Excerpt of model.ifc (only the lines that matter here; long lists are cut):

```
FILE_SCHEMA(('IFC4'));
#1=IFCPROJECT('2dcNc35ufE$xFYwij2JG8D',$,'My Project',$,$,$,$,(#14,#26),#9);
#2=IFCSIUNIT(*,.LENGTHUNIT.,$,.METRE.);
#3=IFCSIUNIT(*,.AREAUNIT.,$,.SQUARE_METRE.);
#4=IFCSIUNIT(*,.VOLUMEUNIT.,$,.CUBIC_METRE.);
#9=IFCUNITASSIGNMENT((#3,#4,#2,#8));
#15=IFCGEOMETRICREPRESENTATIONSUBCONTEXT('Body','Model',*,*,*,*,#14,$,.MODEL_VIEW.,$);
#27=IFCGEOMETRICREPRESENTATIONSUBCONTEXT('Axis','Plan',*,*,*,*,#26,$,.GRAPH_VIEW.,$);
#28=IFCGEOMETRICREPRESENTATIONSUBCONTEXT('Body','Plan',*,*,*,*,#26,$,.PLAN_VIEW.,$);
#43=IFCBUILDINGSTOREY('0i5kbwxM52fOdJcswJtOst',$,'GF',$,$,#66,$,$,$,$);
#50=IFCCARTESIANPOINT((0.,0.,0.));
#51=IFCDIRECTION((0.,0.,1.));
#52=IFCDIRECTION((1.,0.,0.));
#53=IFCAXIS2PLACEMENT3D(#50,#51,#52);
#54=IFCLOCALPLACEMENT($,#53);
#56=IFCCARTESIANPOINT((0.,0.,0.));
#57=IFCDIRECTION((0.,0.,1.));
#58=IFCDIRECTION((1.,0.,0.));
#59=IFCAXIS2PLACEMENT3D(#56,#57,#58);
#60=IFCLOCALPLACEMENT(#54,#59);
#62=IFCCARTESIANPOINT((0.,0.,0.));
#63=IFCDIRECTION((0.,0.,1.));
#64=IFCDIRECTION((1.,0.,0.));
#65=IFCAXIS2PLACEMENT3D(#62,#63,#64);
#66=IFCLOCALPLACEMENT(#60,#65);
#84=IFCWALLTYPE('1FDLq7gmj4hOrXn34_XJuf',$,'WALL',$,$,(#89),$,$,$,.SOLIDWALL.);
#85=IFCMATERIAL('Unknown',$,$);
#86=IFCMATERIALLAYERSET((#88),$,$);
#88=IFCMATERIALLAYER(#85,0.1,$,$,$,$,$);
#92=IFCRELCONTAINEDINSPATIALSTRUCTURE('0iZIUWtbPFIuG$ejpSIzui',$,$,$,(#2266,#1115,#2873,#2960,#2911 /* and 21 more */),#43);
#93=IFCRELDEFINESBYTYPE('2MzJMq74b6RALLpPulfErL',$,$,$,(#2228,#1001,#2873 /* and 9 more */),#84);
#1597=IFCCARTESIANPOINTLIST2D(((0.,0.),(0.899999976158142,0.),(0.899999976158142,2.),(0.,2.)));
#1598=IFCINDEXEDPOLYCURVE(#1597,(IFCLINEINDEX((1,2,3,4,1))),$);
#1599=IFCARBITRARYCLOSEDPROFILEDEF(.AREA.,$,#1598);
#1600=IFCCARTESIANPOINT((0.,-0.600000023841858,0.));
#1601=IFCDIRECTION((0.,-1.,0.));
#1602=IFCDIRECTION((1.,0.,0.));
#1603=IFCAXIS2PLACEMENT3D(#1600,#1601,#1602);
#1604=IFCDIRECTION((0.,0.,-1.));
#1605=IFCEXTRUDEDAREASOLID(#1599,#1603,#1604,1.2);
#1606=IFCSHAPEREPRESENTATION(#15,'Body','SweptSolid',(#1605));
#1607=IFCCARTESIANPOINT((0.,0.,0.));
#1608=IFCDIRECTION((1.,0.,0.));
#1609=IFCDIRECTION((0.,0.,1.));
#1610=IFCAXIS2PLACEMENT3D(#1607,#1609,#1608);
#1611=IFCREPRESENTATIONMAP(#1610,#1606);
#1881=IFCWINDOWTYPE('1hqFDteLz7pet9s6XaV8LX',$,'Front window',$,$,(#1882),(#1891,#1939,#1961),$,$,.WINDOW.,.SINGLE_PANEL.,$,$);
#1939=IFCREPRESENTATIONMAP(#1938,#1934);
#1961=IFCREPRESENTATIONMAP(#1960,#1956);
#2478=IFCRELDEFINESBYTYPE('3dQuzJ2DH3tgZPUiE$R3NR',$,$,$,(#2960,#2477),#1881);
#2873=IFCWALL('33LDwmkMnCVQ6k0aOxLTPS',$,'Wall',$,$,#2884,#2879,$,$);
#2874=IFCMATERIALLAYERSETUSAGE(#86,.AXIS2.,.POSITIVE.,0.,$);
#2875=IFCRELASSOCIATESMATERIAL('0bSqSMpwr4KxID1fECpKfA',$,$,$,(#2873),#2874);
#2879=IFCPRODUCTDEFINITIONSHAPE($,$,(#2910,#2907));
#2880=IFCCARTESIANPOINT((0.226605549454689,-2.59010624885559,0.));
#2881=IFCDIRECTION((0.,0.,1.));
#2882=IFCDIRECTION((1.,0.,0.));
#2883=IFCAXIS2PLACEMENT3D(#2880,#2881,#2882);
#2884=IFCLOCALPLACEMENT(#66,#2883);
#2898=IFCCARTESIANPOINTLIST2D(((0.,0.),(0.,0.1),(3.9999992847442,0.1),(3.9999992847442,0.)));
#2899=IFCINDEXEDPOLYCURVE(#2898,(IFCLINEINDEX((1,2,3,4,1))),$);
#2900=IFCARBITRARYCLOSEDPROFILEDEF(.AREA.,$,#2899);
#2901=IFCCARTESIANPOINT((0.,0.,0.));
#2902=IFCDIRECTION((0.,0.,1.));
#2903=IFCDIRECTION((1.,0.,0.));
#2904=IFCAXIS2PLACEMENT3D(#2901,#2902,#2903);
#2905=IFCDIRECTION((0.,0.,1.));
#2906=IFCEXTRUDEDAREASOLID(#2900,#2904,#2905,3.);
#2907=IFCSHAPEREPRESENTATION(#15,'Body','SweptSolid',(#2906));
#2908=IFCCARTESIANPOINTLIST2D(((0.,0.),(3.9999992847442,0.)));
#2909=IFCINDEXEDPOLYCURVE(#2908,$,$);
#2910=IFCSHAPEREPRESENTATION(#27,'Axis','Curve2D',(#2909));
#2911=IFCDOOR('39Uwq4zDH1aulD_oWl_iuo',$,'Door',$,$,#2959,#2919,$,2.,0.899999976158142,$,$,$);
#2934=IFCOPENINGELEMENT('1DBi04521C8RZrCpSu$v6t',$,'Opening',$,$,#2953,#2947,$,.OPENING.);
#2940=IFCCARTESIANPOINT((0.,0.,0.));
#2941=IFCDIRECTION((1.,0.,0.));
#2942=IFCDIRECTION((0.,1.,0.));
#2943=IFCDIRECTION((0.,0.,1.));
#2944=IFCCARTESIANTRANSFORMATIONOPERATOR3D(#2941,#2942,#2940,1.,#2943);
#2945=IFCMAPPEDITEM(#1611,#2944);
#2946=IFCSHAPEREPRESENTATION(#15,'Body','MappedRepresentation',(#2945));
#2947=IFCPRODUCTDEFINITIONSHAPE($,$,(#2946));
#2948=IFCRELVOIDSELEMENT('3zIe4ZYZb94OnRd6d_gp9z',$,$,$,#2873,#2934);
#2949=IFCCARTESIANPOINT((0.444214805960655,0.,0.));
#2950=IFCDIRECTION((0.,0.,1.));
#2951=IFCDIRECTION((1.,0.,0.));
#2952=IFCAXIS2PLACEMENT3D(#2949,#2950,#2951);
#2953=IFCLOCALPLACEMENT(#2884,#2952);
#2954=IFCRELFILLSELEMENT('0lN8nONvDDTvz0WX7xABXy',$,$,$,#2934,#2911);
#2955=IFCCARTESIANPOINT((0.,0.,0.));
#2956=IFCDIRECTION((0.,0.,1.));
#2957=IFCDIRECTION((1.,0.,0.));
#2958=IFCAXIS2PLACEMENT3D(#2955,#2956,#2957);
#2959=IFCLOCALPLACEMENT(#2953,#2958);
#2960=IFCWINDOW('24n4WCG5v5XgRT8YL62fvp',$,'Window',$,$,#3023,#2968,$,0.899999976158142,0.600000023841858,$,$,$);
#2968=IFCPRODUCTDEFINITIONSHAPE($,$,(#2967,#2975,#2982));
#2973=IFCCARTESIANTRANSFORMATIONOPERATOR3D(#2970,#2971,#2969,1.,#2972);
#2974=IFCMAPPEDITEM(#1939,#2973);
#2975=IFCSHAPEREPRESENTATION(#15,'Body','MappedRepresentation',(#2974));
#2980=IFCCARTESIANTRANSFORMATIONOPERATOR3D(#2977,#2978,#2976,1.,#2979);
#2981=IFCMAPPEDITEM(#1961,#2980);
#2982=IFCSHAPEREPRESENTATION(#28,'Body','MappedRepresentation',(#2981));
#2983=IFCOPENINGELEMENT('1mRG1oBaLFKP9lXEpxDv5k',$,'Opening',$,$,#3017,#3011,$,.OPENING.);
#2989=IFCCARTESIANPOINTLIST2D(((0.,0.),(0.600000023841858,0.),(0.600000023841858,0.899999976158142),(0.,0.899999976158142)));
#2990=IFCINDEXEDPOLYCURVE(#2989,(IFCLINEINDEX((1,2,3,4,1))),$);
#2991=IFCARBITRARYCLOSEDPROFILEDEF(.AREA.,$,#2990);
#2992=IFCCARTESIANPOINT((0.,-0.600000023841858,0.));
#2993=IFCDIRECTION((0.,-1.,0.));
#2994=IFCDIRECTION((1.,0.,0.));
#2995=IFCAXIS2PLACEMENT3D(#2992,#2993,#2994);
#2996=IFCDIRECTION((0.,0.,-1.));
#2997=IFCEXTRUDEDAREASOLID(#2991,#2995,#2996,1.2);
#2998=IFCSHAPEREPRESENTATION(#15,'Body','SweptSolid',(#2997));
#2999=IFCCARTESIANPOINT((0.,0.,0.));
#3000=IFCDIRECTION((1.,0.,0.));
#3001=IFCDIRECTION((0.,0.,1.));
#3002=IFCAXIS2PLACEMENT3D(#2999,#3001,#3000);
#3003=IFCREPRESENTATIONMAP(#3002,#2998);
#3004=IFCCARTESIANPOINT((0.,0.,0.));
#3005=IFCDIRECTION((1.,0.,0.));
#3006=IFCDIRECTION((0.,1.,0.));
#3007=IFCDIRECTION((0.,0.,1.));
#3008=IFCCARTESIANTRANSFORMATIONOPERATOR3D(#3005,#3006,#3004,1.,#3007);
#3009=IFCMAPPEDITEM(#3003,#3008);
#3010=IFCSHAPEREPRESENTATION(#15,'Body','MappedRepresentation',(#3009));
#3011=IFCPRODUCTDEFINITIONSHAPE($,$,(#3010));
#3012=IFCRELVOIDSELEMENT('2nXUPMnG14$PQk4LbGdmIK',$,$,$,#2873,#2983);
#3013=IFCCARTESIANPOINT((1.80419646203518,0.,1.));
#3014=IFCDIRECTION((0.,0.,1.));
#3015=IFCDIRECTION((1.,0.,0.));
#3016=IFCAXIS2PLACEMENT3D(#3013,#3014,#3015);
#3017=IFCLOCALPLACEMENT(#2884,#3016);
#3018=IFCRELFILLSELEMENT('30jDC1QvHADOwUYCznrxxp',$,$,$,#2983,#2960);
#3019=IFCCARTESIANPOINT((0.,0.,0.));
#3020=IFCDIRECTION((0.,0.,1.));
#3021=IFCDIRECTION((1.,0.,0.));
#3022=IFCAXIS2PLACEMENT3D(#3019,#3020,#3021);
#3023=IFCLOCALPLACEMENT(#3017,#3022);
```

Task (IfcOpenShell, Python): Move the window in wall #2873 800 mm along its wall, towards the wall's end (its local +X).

```python
import ifcopenshell
import ifcopenshell.api.geometry
import ifcopenshell.util.placement
import ifcopenshell.util.unit

model = ifcopenshell.open("model.ifc")
unit_scale = ifcopenshell.util.unit.calculate_unit_scale(model)

window = model.by_id(2960)
opening = window.FillsVoids[0].RelatingOpeningElement
wall = opening.VoidsElements[0].RelatingBuildingElement

wall_matrix = ifcopenshell.util.placement.get_local_placement(wall.ObjectPlacement)
shift = wall_matrix[:3, 0] * 0.8 / unit_scale
before = ifcopenshell.util.placement.get_local_placement(window.ObjectPlacement)[:3, 3].copy()

# The window is placed relative to its opening, so it follows when the opening moves.
matrix = ifcopenshell.util.placement.get_local_placement(opening.ObjectPlacement)
matrix[:3, 3] += shift
ifcopenshell.api.geometry.edit_object_placement(
    model, product=opening, matrix=matrix, is_si=False, should_transform_children=True
)

after = ifcopenshell.util.placement.get_local_placement(window.ObjectPlacement)[:3, 3]
print("window moved by", (after - before).round(3) + 0.0)

model.write("model_updated.ifc")
```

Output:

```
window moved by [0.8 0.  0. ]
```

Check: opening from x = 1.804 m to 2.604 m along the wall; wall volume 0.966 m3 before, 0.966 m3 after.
